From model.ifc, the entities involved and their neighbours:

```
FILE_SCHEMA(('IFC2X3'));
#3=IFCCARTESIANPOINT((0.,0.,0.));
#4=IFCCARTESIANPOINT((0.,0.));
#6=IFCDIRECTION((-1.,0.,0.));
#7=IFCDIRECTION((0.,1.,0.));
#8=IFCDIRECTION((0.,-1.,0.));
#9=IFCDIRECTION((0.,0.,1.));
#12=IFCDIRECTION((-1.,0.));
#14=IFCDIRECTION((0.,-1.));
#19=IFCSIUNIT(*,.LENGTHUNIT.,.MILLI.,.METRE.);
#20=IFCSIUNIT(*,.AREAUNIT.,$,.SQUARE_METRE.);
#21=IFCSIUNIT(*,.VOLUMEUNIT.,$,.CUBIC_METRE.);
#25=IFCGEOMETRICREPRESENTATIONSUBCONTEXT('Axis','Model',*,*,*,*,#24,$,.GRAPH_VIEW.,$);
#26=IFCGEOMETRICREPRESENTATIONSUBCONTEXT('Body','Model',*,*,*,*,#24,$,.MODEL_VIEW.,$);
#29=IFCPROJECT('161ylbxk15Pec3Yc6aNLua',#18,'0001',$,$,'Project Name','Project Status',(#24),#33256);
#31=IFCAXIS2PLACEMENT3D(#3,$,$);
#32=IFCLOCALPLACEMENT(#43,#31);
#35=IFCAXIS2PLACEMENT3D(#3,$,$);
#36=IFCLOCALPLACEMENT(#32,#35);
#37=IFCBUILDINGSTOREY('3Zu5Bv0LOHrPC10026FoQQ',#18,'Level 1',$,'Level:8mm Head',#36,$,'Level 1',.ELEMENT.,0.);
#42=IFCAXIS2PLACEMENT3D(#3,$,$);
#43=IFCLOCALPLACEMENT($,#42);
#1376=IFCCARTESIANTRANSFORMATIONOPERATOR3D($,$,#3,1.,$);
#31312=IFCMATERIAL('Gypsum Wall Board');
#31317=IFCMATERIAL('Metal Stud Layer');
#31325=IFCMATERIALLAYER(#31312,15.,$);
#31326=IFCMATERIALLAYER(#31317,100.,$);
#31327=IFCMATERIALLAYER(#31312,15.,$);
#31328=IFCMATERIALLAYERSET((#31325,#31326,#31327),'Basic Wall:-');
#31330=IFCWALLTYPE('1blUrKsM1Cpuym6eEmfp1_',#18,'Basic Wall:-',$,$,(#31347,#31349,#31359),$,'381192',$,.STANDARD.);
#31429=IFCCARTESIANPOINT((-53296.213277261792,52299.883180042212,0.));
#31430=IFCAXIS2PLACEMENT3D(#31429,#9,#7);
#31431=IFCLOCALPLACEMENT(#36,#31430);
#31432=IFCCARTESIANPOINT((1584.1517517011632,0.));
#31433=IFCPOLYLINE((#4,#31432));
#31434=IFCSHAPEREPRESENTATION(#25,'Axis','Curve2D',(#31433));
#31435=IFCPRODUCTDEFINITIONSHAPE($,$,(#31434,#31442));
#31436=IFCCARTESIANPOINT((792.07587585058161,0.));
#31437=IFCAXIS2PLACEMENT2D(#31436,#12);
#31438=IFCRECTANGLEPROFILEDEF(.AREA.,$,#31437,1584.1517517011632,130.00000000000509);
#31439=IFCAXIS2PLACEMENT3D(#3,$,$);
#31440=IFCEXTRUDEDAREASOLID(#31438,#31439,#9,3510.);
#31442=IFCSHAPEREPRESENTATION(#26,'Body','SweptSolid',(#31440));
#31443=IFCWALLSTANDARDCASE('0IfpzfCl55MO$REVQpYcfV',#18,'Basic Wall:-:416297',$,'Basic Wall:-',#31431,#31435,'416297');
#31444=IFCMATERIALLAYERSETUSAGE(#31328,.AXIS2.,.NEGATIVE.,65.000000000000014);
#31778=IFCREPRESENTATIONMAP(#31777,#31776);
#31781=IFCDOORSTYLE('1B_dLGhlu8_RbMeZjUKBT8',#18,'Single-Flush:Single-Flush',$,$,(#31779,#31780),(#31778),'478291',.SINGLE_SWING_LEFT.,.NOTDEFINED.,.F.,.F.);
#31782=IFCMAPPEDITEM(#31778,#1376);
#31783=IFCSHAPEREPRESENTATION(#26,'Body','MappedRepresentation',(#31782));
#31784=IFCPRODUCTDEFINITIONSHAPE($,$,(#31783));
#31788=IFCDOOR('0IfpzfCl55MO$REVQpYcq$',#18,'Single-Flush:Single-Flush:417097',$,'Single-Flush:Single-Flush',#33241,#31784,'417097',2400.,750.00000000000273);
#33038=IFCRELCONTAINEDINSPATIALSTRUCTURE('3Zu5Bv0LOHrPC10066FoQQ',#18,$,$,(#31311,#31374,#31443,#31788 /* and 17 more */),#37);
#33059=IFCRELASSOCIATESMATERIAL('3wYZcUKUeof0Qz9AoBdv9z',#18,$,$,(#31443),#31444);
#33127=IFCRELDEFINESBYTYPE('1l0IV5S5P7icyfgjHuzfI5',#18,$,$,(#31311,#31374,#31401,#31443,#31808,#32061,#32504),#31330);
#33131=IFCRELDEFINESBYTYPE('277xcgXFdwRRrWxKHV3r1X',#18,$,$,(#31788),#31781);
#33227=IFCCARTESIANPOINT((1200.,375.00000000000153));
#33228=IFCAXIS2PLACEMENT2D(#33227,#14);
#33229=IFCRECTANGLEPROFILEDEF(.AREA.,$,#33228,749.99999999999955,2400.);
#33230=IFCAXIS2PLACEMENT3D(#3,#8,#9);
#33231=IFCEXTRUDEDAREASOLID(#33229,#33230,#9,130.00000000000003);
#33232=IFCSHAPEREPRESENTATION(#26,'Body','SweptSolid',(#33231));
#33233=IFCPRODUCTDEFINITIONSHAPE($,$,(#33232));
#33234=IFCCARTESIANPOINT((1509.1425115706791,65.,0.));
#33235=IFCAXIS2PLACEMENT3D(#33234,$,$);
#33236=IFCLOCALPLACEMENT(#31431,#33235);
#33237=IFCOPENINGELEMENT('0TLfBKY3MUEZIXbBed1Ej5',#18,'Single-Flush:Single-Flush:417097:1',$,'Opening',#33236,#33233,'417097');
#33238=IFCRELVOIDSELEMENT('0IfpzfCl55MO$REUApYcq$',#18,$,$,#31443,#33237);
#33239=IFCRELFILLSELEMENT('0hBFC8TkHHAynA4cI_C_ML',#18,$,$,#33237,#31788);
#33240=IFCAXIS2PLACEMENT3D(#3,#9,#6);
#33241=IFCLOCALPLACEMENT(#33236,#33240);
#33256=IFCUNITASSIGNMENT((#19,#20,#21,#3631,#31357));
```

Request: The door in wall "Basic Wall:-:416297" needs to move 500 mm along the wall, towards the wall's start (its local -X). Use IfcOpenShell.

```python
import ifcopenshell
import ifcopenshell.api.geometry
import ifcopenshell.util.placement
import ifcopenshell.util.unit

model = ifcopenshell.open("model.ifc")
unit_scale = ifcopenshell.util.unit.calculate_unit_scale(model)

door = model.by_guid("0IfpzfCl55MO$REVQpYcq$")
opening = door.FillsVoids[0].RelatingOpeningElement
wall = opening.VoidsElements[0].RelatingBuildingElement

wall_matrix = ifcopenshell.util.placement.get_local_placement(wall.ObjectPlacement)
shift = wall_matrix[:3, 0] * -0.5 / unit_scale
before = ifcopenshell.util.placement.get_local_placement(door.ObjectPlacement)[:3, 3].copy()

# The door is placed relative to its opening, so it follows when the opening moves.
matrix = ifcopenshell.util.placement.get_local_placement(opening.ObjectPlacement)
matrix[:3, 3] += shift
ifcopenshell.api.geometry.edit_object_placement(
    model, product=opening, matrix=matrix, is_si=False, should_transform_children=True
)

after = ifcopenshell.util.placement.get_local_placement(door.ObjectPlacement)[:3, 3]
print("door moved by", (after - before).round(3) + 0.0)

model.write("model_v2.ifc")
```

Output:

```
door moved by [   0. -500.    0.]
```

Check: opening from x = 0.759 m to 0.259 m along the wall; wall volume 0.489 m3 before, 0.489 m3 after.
